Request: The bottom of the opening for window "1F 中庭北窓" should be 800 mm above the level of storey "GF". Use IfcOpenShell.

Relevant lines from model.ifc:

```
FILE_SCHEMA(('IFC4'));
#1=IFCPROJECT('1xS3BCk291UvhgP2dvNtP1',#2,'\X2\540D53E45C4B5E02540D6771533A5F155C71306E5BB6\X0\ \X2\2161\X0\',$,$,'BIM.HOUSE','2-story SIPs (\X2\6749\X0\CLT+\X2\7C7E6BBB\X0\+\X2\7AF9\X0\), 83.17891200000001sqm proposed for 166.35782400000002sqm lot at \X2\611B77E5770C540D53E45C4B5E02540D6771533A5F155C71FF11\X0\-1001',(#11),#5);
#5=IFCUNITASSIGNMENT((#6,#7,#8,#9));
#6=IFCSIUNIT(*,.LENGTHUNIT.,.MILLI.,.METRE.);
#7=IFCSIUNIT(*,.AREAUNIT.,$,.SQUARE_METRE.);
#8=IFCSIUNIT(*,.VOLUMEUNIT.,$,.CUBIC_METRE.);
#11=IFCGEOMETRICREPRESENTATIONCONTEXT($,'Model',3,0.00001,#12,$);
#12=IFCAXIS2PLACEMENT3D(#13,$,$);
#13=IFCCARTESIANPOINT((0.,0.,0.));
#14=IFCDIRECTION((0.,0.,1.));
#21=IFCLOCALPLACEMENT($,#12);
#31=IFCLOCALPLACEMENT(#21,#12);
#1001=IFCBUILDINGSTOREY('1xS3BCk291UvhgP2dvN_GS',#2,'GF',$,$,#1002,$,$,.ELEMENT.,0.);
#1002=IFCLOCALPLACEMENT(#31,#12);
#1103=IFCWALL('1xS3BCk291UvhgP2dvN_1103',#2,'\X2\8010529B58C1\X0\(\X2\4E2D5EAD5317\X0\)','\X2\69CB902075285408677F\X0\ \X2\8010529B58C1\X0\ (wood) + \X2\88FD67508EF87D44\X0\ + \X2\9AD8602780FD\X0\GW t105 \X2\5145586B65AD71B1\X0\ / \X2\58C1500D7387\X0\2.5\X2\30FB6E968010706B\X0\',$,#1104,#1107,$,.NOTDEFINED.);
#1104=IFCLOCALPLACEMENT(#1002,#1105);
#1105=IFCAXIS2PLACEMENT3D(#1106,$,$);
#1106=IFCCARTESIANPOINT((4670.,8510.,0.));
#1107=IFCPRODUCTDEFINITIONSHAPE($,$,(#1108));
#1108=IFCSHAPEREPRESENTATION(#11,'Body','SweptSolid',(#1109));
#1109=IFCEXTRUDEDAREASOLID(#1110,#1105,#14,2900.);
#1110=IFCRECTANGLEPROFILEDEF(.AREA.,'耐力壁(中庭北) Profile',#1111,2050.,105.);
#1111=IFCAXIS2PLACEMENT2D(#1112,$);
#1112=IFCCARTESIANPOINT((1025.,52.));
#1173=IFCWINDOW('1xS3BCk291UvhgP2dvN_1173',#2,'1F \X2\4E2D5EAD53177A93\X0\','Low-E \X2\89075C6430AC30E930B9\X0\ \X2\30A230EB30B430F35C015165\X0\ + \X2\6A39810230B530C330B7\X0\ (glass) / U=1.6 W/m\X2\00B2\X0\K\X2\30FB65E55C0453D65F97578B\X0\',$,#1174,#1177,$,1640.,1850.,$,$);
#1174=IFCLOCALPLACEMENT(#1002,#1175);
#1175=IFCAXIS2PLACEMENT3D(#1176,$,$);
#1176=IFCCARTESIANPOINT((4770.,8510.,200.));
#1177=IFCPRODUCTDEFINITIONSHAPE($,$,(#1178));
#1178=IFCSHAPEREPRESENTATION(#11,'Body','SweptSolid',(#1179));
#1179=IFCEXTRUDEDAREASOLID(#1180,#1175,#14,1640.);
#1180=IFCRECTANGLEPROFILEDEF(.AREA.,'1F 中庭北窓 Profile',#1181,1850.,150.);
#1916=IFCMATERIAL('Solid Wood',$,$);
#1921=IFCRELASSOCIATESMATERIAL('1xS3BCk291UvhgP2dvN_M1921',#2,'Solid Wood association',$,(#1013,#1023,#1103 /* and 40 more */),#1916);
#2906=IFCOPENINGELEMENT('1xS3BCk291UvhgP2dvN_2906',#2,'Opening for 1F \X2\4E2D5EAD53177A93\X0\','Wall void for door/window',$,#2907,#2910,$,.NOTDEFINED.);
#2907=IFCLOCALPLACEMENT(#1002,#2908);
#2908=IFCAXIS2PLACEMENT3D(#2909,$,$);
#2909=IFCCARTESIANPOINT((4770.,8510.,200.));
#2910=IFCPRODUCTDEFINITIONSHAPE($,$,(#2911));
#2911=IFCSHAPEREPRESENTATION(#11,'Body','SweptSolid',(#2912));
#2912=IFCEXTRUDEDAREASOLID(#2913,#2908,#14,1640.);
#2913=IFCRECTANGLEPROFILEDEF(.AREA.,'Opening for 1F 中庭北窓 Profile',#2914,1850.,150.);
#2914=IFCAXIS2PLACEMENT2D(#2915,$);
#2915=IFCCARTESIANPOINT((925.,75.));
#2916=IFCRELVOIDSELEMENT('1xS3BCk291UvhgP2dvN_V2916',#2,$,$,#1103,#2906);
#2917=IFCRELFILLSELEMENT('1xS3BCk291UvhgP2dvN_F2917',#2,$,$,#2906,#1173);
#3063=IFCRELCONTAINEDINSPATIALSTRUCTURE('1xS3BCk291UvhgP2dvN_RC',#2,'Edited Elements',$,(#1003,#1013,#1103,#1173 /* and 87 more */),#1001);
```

```python
import numpy as np
import ifcopenshell
import ifcopenshell.api.geometry
import ifcopenshell.geom
import ifcopenshell.util.element
import ifcopenshell.util.placement
import ifcopenshell.util.shape
import ifcopenshell.util.unit

model = ifcopenshell.open("model.ifc")
unit_scale = ifcopenshell.util.unit.calculate_unit_scale(model)

window = model.by_guid("1xS3BCk291UvhgP2dvN_1173")
opening = window.FillsVoids[0].RelatingOpeningElement
storey = ifcopenshell.util.element.get_container(window, ifc_class="IfcBuildingStorey")
level = ifcopenshell.util.placement.get_local_placement(storey.ObjectPlacement)[2, 3]

# The opening's origin need not be at the sill, so measure its lowest point.
shape = ifcopenshell.geom.create_shape(ifcopenshell.geom.settings(), opening)
bottom = ifcopenshell.util.shape.get_shape_bottom_elevation(shape, shape.geometry) / unit_scale
dz = level + 0.8 / unit_scale - bottom

shift = np.array([0.0, 0.0, dz])
# The window is not placed relative to its opening, so move both.
for product in (opening, window):
    matrix = ifcopenshell.util.placement.get_local_placement(product.ObjectPlacement)
    matrix[:3, 3] += shift
    ifcopenshell.api.geometry.edit_object_placement(model, product=product, matrix=matrix, is_si=False)

print(f"moved by {dz * unit_scale:+.3f} m")

model.write("model_rev.ifc")
```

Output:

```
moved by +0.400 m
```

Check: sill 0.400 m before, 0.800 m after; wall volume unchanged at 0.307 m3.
